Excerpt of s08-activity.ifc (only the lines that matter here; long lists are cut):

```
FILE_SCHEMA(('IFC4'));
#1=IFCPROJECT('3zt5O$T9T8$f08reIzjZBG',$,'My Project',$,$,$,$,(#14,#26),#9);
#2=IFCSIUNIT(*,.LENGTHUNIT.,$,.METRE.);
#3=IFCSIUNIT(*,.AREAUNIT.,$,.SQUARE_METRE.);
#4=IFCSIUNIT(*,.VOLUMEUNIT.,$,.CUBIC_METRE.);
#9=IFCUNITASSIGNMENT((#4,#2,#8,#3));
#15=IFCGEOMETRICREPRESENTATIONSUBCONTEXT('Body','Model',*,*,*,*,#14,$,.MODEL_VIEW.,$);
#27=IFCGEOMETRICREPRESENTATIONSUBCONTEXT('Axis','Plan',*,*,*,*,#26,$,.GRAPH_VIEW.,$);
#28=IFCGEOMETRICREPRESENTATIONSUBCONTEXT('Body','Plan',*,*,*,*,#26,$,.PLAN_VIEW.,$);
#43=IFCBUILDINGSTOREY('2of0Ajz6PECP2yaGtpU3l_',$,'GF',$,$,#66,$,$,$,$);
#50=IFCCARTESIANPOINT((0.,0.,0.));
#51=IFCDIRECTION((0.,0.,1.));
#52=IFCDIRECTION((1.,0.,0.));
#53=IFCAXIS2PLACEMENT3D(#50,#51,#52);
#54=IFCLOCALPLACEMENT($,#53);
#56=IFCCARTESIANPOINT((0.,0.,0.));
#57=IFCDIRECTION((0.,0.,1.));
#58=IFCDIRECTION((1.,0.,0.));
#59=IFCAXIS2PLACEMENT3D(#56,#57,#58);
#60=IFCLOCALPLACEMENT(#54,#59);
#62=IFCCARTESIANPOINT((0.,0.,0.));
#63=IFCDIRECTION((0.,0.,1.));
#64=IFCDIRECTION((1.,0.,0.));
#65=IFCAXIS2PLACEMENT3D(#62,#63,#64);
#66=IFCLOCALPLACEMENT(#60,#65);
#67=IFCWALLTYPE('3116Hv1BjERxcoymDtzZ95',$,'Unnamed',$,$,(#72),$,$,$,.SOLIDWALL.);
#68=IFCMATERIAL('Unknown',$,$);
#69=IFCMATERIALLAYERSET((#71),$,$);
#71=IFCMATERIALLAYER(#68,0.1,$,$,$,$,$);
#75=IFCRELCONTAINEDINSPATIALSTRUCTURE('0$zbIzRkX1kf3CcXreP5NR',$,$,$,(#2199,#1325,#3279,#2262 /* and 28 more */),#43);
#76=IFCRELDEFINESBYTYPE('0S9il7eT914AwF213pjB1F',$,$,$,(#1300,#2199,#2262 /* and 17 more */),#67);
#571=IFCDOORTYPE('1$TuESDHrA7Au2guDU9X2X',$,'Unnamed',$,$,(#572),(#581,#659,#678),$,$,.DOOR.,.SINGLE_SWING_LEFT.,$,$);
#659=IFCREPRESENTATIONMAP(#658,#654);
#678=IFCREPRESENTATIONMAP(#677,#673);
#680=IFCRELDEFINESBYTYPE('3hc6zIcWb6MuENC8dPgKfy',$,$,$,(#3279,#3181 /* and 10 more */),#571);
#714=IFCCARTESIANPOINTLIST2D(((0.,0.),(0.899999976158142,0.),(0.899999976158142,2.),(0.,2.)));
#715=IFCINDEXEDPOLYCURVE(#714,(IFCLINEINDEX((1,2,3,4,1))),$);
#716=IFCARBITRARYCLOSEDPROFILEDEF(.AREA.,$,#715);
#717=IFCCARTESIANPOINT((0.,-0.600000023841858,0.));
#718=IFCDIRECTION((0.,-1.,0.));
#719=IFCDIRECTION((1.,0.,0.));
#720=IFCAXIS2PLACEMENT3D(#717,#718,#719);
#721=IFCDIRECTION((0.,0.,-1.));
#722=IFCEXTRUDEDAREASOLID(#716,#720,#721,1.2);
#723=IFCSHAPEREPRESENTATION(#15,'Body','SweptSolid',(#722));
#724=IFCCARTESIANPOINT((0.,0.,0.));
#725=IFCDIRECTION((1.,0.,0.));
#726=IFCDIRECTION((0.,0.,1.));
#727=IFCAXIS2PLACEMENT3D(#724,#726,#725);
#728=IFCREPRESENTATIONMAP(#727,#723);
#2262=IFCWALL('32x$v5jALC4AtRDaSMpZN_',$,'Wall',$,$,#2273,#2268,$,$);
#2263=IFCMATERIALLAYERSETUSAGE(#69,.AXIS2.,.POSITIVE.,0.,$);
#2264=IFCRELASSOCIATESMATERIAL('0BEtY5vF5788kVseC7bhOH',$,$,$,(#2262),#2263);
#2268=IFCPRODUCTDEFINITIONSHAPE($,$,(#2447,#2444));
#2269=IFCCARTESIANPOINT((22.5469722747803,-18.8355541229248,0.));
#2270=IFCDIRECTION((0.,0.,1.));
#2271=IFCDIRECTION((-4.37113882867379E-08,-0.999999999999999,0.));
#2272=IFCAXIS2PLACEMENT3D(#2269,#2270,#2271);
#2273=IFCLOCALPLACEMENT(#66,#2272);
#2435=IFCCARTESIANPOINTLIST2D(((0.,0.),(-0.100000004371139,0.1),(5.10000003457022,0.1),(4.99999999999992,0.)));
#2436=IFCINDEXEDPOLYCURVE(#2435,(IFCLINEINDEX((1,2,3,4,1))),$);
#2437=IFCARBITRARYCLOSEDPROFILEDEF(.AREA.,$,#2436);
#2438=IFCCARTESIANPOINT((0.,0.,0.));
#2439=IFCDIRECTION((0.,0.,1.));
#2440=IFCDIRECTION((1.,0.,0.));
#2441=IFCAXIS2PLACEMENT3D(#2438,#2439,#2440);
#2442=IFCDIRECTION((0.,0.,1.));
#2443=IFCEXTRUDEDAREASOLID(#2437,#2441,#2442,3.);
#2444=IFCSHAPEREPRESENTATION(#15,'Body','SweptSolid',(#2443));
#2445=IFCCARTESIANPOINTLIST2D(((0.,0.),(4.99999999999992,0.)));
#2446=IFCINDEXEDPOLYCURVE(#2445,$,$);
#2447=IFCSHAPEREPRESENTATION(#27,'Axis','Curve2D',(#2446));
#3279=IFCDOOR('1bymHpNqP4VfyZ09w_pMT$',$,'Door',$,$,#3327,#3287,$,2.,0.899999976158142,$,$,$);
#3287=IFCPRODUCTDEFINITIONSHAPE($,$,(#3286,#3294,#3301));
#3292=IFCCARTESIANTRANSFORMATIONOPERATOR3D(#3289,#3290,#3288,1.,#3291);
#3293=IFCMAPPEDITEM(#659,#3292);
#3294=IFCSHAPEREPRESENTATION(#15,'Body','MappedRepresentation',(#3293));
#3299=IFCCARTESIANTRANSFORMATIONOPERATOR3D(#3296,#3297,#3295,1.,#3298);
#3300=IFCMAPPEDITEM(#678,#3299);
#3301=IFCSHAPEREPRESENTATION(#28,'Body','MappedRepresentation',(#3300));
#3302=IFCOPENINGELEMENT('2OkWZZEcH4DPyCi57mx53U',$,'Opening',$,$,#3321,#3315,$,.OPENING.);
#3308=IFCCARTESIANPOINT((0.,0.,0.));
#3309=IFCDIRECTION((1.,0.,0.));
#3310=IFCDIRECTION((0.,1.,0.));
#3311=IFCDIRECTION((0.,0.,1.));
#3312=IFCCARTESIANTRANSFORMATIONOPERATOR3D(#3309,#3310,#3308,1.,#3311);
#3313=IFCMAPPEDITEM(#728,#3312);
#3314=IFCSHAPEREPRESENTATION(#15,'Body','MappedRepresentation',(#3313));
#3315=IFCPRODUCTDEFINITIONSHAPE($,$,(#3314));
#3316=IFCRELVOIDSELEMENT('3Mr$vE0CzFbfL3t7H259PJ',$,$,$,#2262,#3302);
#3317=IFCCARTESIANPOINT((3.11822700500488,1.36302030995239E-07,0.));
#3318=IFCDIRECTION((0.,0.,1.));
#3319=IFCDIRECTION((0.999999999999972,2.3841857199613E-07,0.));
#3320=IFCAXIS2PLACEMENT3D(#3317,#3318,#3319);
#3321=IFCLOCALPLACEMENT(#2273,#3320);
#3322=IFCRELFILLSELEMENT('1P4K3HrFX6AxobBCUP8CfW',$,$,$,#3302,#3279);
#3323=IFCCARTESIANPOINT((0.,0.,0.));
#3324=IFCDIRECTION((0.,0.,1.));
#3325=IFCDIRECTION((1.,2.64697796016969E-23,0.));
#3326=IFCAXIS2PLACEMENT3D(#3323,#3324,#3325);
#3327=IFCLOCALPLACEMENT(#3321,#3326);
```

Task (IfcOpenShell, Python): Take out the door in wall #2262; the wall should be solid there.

```python
import ifcopenshell
import ifcopenshell.api.feature
import ifcopenshell.api.root
import ifcopenshell.geom
import ifcopenshell.util.shape

model = ifcopenshell.open("s08-activity.ifc")
settings = ifcopenshell.geom.settings()


def volume(element):
    """Net volume in cubic metres, openings subtracted."""
    shape = ifcopenshell.geom.create_shape(settings, element)
    return ifcopenshell.util.shape.get_volume(shape.geometry)


door = model.by_guid("1bymHpNqP4VfyZ09w_pMT$")
opening = door.FillsVoids[0].RelatingOpeningElement
wall = opening.VoidsElements[0].RelatingBuildingElement
before = volume(wall)

ifcopenshell.api.root.remove_product(model, product=door)
ifcopenshell.api.feature.remove_feature(model, feature=opening)

after = volume(wall)

print(f"wall volume {before:.3f} -> {after:.3f} m3")

model.write("s08-activity_updated.ifc")
```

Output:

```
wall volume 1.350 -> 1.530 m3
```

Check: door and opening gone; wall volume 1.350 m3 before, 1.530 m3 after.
